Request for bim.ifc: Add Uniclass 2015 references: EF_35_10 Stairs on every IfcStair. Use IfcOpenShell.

First a look at what the model holds.

```python
import ifcopenshell

model = ifcopenshell.open("bim.ifc")
print(model.schema)
print("classifications:", [c.Name for c in model.by_type("IfcClassification")])
for ifc_class in ("IfcDoor", "IfcRoof", "IfcStair", "IfcWall", "IfcWindow"):
    print(ifc_class, len(model.by_type(ifc_class)))
```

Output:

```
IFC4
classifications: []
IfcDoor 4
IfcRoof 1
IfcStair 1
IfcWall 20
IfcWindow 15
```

```python
import ifcopenshell
import ifcopenshell.api.classification

model = ifcopenshell.open("bim.ifc")

system = ifcopenshell.api.classification.add_classification(model, classification="Uniclass 2015")

codes = {
    "IfcStair": ("EF_35_10", "Stairs"),
}
for ifc_class, (code, name) in codes.items():
    products = model.by_type(ifc_class)
    ifcopenshell.api.classification.add_reference(
        model, products=products, classification=system, identification=code, name=name
    )
    print(code, len(products))

model.write("bim_edited.ifc")
```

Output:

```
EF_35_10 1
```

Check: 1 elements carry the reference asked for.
